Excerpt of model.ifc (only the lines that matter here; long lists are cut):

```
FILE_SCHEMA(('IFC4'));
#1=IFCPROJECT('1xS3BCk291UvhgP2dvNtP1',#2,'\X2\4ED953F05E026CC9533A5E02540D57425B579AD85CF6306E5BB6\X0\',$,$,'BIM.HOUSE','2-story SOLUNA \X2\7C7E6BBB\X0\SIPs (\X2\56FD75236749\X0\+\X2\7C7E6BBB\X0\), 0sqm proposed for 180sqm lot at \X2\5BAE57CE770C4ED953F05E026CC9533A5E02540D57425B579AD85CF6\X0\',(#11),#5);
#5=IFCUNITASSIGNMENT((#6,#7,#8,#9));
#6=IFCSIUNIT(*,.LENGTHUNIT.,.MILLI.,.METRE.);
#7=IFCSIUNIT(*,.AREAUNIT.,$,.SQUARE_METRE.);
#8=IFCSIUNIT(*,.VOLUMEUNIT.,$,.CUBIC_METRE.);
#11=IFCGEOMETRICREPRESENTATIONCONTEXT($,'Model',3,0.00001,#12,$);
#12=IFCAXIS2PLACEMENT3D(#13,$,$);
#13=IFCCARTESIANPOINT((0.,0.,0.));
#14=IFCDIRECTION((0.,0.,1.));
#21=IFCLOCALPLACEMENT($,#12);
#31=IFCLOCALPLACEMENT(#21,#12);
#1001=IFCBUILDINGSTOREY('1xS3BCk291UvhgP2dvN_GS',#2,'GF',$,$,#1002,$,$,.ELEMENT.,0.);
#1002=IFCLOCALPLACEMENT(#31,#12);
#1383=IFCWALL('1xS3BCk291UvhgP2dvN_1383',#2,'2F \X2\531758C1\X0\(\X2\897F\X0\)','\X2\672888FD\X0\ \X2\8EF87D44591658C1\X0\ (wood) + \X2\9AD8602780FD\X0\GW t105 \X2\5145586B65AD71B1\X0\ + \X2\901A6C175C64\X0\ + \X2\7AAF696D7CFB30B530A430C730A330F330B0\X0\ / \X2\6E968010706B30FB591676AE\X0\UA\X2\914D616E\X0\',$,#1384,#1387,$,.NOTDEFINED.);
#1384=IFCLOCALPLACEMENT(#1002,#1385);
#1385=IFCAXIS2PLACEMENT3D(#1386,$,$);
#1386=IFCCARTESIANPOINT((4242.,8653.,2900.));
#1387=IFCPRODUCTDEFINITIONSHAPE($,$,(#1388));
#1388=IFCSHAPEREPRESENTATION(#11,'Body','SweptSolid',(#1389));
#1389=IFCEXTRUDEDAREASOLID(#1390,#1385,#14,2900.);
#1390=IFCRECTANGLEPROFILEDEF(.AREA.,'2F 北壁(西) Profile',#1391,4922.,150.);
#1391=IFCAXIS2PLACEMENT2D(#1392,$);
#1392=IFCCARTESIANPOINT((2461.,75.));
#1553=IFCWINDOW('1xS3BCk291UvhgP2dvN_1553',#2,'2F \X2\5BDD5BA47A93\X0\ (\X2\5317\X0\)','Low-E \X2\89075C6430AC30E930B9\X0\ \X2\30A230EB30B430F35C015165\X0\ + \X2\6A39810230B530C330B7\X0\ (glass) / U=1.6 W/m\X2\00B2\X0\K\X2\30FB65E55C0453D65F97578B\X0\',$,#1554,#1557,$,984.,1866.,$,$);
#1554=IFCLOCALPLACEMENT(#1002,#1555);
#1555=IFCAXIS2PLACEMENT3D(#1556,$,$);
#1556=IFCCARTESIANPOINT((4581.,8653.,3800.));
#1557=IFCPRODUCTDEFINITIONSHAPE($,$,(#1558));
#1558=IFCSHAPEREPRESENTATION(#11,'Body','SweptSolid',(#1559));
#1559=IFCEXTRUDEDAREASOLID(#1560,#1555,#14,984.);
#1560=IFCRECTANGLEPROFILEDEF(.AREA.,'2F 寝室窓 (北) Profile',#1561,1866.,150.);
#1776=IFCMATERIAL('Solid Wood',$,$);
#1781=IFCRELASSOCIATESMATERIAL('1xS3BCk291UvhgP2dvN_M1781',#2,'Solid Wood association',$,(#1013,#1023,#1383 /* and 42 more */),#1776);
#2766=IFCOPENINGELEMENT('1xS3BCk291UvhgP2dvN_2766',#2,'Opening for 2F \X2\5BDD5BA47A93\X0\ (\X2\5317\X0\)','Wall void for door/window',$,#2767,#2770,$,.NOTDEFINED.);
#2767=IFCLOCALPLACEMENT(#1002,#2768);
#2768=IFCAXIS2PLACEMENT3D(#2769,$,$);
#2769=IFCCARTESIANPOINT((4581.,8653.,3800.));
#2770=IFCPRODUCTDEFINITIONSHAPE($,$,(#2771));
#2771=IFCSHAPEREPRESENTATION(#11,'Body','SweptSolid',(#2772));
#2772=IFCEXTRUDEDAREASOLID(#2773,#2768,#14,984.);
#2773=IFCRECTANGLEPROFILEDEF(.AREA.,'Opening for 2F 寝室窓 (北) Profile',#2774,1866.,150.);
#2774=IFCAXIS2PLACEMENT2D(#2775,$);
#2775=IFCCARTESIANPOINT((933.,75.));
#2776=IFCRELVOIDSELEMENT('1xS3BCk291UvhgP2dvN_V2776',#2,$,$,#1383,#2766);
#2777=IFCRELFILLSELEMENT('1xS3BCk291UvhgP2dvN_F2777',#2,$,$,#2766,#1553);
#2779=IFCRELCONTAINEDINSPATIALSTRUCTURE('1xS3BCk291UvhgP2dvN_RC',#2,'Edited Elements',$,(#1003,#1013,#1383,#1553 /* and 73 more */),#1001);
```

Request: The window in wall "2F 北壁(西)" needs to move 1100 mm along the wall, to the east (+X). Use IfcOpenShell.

```python
import ifcopenshell
import ifcopenshell.api.geometry
import ifcopenshell.util.placement

model = ifcopenshell.open("model.ifc")

window = model.by_guid("1xS3BCk291UvhgP2dvN_1553")
opening = window.FillsVoids[0].RelatingOpeningElement
wall = opening.VoidsElements[0].RelatingBuildingElement

wall_matrix = ifcopenshell.util.placement.get_local_placement(wall.ObjectPlacement)
shift = wall_matrix[:3, 0] * 1100.0
before = ifcopenshell.util.placement.get_local_placement(window.ObjectPlacement)[:3, 3].copy()

# The window is not placed relative to its opening, so move both.
for product in (opening, window):
    matrix = ifcopenshell.util.placement.get_local_placement(product.ObjectPlacement)
    matrix[:3, 3] += shift
    ifcopenshell.api.geometry.edit_object_placement(model, product=product, matrix=matrix, is_si=False)

after = ifcopenshell.util.placement.get_local_placement(window.ObjectPlacement)[:3, 3]
print("window moved by", (after - before).round(3) + 0.0)

model.write("model_edited.ifc")
```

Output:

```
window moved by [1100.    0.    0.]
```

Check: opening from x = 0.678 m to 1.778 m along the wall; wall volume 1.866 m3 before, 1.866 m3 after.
